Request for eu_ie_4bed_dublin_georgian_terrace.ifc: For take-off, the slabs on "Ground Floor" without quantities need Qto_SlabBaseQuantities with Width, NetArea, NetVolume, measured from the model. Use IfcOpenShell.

First a look at what the model holds.

```python
import ifcopenshell
import ifcopenshell.util.element
import ifcopenshell.util.unit

model = ifcopenshell.open("eu_ie_4bed_dublin_georgian_terrace.ifc")
print(model.schema)
for unit_type in ("LENGTHUNIT", "AREAUNIT", "VOLUMEUNIT"):
    print(unit_type, ifcopenshell.util.unit.calculate_unit_scale(model, unit_type))
storey = next(s for s in model.by_type("IfcBuildingStorey") if s.Name == "Ground Floor")
slabs = [e for e in ifcopenshell.util.element.get_decomposition(storey) if e.is_a("IfcSlab")]
for e in sorted(slabs, key=lambda e: e.id()):
    print(e.id(), e.is_a(), e.Name, list(ifcopenshell.util.element.get_psets(e, qtos_only=True)), sep=" | ")
```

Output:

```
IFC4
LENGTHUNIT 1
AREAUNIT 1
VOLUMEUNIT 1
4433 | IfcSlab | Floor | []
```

```python
import ifcopenshell
import ifcopenshell.api.pset
import ifcopenshell.geom
import ifcopenshell.util.element
import ifcopenshell.util.shape
import ifcopenshell.util.unit

model = ifcopenshell.open("eu_ie_4bed_dublin_georgian_terrace.ifc")
unit_scale = ifcopenshell.util.unit.calculate_unit_scale(model)
area_scale = ifcopenshell.util.unit.calculate_unit_scale(model, "AREAUNIT")
volume_scale = ifcopenshell.util.unit.calculate_unit_scale(model, "VOLUMEUNIT")
settings = ifcopenshell.geom.settings()

storey = next(s for s in model.by_type("IfcBuildingStorey") if s.Name == "Ground Floor")
slabs = [e for e in ifcopenshell.util.element.get_decomposition(storey) if e.is_a("IfcSlab")]

for e in sorted(slabs, key=lambda e: e.id()):
    if ifcopenshell.util.element.get_psets(e, qtos_only=True, should_inherit=False):
        continue
    # Geometry comes back in metres, in the element's own axes.
    shape = ifcopenshell.geom.create_shape(settings, e)
    values = {
        "Width": ifcopenshell.util.shape.get_z(shape.geometry) / unit_scale,
        "NetArea": ifcopenshell.util.shape.get_footprint_area(shape.geometry) / area_scale,
        "NetVolume": ifcopenshell.util.shape.get_volume(shape.geometry) / volume_scale,
    }
    qto = ifcopenshell.api.pset.add_qto(model, product=e, name="Qto_SlabBaseQuantities")
    ifcopenshell.api.pset.edit_qto(model, qto=qto, properties=values)
    print(e.id(), {k: round(v, 3) for k, v in values.items()})

model.write("eu_ie_4bed_dublin_georgian_terrace_edited.ifc")
```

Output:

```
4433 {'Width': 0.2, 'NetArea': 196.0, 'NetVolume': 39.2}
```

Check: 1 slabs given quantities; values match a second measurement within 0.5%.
